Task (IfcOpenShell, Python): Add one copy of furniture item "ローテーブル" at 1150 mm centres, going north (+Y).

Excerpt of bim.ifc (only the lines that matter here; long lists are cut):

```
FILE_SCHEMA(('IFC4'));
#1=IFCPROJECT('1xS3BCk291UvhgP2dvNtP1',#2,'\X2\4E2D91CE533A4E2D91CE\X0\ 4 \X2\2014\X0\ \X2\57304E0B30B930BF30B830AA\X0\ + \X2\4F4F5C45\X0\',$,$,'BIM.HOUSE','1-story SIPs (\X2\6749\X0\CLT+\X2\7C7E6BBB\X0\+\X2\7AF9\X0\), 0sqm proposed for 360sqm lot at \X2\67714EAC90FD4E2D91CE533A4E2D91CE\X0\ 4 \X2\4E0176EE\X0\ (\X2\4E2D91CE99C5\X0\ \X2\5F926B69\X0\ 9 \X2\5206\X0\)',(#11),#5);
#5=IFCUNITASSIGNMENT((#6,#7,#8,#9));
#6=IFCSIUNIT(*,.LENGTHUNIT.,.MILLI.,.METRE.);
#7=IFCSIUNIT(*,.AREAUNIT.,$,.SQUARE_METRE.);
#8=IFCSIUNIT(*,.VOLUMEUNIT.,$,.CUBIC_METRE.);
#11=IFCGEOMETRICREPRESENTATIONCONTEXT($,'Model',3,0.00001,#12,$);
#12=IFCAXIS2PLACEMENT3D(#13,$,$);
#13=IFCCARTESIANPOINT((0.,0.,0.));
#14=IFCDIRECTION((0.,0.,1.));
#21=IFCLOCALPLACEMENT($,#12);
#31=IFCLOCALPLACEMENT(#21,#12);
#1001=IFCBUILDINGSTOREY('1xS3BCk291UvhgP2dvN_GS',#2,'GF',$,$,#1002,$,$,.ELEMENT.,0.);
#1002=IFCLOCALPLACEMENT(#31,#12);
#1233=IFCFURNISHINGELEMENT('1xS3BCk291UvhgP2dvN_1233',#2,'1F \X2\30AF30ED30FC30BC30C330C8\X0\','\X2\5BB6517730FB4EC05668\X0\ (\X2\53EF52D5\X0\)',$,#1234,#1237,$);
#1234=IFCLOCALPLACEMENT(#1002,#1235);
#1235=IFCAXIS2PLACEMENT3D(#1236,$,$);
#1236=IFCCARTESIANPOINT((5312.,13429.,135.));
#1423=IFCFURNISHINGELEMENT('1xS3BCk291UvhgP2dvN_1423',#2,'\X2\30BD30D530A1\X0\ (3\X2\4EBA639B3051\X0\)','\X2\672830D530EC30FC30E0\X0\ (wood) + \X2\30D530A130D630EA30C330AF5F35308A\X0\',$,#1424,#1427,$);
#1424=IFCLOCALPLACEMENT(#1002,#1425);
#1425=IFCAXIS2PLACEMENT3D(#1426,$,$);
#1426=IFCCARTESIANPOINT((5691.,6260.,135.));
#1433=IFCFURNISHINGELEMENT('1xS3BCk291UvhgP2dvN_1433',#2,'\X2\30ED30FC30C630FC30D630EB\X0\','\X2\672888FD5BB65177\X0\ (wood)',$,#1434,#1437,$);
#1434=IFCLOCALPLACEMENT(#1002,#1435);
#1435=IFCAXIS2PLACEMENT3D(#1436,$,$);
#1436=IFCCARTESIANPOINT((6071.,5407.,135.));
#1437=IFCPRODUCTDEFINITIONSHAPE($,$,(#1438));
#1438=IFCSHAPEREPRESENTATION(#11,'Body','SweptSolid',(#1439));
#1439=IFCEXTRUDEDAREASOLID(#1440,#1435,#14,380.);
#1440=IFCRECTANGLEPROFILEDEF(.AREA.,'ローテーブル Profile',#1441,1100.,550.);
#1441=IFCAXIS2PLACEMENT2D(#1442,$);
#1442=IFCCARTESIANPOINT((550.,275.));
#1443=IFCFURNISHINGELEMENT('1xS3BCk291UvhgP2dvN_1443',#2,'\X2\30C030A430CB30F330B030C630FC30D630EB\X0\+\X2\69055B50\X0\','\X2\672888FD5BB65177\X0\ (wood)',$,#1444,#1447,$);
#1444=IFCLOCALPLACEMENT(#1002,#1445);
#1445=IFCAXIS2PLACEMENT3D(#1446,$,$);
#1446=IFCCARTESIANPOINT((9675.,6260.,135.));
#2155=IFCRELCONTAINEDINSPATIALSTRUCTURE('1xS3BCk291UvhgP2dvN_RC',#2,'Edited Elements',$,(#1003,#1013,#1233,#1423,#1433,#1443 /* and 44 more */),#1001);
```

```python
import numpy as np
import ifcopenshell
import ifcopenshell.api.geometry
import ifcopenshell.api.root
import ifcopenshell.util.element
import ifcopenshell.util.placement

model = ifcopenshell.open("bim.ifc")


def reuse_history(source, copy):
    """copy_class also copies each property set's owner history, people and application; keep the originals."""
    for rel in copy.IsDefinedBy:
        if rel.is_a("IfcRelDefinesByProperties") and (history := rel.RelatingPropertyDefinition.OwnerHistory):
            rel.RelatingPropertyDefinition.OwnerHistory = source.OwnerHistory
            ifcopenshell.util.element.remove_deep2(model, history)


source = model.by_id(1433)
base = ifcopenshell.util.placement.get_local_placement(source.ObjectPlacement)
step = np.array([0.0, 1.0, 0.0]) * 1150.0

for i in range(1, 2):
    copy = ifcopenshell.api.root.copy_class(model, product=source)
    copy.Representation = ifcopenshell.util.element.copy_deep(
        model, source.Representation, exclude=["IfcGeometricRepresentationContext", "IfcRepresentationMap"]
    )
    reuse_history(source, copy)
    matrix = base.copy()
    matrix[:3, 3] += i * step
    print("added at", matrix[:3, 3].round(3) + 0.0)
    ifcopenshell.api.geometry.edit_object_placement(model, product=copy, matrix=matrix, is_si=False)

model.write("bim-out.ifc")
```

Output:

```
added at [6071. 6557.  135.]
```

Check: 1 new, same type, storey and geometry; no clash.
